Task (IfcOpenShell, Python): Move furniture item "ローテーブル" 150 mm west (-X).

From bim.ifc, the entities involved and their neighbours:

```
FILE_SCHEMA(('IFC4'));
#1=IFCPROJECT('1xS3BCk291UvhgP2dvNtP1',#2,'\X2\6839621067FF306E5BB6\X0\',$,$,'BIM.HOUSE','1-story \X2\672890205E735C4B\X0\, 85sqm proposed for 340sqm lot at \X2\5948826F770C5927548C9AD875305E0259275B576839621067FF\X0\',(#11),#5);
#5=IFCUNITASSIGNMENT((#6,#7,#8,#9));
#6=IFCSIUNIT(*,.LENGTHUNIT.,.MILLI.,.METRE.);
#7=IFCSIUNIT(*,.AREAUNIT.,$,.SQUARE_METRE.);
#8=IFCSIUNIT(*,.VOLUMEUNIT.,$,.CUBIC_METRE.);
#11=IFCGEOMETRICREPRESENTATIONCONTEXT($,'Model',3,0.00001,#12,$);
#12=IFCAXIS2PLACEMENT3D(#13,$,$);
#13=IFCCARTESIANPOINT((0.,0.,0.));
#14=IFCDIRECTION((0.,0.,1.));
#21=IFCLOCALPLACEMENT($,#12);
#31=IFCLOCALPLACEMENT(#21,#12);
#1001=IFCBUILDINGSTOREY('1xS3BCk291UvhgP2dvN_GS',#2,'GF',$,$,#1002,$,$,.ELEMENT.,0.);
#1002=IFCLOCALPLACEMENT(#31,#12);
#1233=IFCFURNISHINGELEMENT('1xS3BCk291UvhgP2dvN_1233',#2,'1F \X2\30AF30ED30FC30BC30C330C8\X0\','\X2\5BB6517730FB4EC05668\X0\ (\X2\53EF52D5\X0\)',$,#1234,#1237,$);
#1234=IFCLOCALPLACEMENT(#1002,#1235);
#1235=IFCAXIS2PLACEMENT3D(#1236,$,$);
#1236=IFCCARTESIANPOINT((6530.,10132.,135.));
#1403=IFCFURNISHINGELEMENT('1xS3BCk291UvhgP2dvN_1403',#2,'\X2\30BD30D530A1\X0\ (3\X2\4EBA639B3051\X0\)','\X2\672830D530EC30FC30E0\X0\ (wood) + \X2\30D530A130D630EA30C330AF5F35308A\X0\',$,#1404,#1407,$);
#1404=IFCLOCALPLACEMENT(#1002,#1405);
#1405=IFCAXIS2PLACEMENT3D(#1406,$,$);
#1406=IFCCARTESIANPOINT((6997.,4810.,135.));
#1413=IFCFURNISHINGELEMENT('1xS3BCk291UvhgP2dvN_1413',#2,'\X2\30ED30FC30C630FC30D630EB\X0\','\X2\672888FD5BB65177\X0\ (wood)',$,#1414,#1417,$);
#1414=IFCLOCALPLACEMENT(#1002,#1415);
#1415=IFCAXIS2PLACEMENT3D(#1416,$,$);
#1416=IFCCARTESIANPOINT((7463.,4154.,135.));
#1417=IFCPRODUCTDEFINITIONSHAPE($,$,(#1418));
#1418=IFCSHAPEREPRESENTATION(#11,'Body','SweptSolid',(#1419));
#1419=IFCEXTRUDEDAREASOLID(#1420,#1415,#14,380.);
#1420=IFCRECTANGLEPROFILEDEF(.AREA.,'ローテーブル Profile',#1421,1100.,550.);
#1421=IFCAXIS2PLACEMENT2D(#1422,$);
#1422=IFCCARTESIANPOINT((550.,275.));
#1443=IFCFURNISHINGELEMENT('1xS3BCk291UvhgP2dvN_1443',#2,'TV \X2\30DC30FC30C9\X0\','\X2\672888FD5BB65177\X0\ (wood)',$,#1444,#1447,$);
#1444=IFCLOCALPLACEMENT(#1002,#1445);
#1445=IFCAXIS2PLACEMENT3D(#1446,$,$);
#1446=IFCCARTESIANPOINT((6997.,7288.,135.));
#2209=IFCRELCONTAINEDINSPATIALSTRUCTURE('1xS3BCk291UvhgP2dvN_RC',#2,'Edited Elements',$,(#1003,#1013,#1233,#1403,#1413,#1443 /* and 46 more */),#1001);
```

```python
import ifcopenshell
import ifcopenshell.api.geometry
import ifcopenshell.util.placement

model = ifcopenshell.open("bim.ifc")

item = model.by_guid("1xS3BCk291UvhgP2dvN_1413")
matrix = ifcopenshell.util.placement.get_local_placement(item.ObjectPlacement)
matrix[0, 3] -= 150.0
ifcopenshell.api.geometry.edit_object_placement(model, product=item, matrix=matrix, is_si=False)

print(ifcopenshell.util.placement.get_local_placement(item.ObjectPlacement).round(3) + 0.0)

model.write("bim_edited.ifc")
```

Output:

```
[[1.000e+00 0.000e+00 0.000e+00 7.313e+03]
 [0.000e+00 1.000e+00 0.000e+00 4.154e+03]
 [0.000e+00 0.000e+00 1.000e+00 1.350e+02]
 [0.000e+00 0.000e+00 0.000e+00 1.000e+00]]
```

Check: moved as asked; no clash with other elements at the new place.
